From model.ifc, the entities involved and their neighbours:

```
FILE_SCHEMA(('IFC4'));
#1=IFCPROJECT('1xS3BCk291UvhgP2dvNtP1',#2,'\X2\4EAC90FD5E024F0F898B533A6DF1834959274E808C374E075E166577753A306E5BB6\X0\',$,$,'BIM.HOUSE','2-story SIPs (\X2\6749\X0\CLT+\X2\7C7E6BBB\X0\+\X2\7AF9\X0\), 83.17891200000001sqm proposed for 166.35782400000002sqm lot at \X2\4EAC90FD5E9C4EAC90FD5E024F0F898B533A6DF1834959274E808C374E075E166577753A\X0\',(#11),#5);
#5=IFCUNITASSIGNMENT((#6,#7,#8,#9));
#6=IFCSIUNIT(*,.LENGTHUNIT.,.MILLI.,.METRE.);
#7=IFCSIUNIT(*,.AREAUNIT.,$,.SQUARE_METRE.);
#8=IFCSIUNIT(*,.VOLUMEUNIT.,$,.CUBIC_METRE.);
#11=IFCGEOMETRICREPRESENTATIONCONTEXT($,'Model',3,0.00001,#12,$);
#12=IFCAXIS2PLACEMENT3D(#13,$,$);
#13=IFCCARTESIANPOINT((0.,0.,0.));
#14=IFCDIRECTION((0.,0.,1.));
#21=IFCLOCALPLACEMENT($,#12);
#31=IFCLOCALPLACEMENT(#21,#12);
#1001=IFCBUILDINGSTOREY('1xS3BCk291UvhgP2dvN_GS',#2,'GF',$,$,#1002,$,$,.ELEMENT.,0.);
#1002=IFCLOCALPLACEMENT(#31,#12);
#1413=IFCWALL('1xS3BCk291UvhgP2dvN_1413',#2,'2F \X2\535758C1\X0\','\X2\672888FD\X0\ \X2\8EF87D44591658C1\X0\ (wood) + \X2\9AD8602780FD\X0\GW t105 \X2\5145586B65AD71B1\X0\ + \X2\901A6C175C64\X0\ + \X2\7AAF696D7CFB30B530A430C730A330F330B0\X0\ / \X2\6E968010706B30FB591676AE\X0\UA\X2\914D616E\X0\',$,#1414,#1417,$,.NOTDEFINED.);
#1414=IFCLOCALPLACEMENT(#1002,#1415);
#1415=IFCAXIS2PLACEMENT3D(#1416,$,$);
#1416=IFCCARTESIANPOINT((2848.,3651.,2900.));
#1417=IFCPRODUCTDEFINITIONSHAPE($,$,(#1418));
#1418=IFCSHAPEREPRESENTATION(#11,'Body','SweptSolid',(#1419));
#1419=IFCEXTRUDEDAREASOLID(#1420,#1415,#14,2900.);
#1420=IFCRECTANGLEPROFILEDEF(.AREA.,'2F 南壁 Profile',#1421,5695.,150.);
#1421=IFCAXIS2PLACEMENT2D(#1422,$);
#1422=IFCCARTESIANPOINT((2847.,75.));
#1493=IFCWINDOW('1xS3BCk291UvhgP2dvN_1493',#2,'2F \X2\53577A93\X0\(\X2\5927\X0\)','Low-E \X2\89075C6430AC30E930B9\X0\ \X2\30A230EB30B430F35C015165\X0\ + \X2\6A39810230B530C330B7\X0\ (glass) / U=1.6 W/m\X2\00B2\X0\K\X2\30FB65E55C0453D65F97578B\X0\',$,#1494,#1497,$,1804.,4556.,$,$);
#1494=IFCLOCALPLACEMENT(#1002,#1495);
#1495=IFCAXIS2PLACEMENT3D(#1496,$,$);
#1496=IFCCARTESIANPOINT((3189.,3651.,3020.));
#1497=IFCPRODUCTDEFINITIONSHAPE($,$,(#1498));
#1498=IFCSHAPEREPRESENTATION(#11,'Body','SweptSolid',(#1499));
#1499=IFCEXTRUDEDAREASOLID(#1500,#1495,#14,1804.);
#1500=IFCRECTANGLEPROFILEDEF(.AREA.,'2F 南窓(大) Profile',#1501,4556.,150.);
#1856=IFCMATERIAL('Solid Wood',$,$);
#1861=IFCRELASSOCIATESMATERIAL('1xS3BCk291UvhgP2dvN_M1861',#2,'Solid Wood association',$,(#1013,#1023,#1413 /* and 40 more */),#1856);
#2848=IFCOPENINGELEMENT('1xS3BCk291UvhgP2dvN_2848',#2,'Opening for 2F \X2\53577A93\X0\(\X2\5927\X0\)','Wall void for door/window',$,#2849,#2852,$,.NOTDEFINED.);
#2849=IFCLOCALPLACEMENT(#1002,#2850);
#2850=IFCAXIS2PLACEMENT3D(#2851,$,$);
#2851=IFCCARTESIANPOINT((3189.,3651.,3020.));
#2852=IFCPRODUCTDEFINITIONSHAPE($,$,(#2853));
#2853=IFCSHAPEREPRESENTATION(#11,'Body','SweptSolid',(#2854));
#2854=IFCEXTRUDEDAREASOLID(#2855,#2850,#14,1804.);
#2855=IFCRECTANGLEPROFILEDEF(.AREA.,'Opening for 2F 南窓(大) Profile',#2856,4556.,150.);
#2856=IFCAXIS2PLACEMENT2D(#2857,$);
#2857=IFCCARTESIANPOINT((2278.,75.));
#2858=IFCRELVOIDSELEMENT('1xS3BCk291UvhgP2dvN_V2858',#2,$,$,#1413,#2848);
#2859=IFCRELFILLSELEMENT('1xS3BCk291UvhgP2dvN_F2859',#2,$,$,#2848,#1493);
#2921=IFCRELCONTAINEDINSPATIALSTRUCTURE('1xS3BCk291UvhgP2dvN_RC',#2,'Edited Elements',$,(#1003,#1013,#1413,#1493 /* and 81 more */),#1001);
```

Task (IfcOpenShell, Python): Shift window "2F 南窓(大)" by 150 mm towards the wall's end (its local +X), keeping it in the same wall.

```python
import ifcopenshell
import ifcopenshell.api.geometry
import ifcopenshell.util.placement

model = ifcopenshell.open("model.ifc")

window = model.by_guid("1xS3BCk291UvhgP2dvN_1493")
opening = window.FillsVoids[0].RelatingOpeningElement
wall = opening.VoidsElements[0].RelatingBuildingElement

wall_matrix = ifcopenshell.util.placement.get_local_placement(wall.ObjectPlacement)
shift = wall_matrix[:3, 0] * 150.0
before = ifcopenshell.util.placement.get_local_placement(window.ObjectPlacement)[:3, 3].copy()

# The window is not placed relative to its opening, so move both.
for product in (opening, window):
    matrix = ifcopenshell.util.placement.get_local_placement(product.ObjectPlacement)
    matrix[:3, 3] += shift
    ifcopenshell.api.geometry.edit_object_placement(model, product=product, matrix=matrix, is_si=False)

after = ifcopenshell.util.placement.get_local_placement(window.ObjectPlacement)[:3, 3]
print("window moved by", (after - before).round(3) + 0.0)

model.write("model_rev.ifc")
```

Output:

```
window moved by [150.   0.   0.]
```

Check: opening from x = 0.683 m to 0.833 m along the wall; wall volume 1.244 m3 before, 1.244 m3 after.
